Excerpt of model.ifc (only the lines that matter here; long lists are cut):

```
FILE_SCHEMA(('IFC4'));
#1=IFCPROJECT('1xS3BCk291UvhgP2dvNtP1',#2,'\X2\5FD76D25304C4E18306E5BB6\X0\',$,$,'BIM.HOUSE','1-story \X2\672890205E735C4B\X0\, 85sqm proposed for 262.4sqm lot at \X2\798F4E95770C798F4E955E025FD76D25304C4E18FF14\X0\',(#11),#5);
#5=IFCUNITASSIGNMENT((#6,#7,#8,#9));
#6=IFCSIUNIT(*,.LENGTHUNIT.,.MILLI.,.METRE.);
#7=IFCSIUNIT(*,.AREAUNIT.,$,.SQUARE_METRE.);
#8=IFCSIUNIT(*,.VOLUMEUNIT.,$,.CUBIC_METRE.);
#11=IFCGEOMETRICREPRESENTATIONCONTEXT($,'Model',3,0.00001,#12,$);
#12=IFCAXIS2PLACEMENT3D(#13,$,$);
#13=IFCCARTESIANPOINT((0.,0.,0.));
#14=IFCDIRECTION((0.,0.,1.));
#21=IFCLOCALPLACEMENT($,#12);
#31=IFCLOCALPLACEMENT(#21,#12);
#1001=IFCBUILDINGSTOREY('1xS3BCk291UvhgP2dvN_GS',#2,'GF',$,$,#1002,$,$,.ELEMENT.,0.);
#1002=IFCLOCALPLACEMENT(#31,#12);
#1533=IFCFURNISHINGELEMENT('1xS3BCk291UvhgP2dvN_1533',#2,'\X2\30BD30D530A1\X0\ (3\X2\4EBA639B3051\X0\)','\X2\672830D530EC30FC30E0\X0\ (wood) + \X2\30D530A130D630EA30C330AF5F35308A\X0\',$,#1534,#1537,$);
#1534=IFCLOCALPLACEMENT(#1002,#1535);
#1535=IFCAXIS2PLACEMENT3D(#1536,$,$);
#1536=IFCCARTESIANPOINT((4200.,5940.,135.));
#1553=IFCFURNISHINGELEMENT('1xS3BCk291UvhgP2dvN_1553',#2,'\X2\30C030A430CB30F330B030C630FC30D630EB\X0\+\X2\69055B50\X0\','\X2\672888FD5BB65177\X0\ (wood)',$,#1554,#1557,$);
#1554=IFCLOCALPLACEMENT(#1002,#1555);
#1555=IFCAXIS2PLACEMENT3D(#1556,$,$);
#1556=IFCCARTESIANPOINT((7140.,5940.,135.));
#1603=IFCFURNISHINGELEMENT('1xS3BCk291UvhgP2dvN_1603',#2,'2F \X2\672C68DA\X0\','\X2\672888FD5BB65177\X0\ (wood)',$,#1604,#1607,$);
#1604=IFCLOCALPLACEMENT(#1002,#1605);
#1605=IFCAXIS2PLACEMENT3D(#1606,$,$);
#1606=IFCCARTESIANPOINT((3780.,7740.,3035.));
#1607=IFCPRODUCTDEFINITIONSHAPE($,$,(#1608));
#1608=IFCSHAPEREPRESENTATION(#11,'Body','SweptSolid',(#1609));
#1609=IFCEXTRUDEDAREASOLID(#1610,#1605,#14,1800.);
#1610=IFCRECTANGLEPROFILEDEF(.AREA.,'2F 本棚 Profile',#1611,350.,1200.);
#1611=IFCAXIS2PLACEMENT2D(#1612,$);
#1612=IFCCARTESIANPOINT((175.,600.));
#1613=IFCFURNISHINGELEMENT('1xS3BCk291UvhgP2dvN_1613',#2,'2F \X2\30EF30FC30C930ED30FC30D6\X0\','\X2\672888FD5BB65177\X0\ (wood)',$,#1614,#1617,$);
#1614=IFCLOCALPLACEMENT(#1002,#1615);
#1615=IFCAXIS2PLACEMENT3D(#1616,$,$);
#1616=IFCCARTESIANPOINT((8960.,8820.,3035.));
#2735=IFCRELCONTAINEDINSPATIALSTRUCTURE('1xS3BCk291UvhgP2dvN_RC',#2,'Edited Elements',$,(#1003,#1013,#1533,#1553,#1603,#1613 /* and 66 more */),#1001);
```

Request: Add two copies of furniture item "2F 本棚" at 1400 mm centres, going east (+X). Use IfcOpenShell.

```python
import numpy as np
import ifcopenshell
import ifcopenshell.api.geometry
import ifcopenshell.api.root
import ifcopenshell.util.element
import ifcopenshell.util.placement
import ifcopenshell.util.unit

model = ifcopenshell.open("model.ifc")
unit_scale = ifcopenshell.util.unit.calculate_unit_scale(model)


def reuse_history(source, copy):
    """copy_class also copies each property set's owner history, people and application; keep the originals."""
    for rel in copy.IsDefinedBy:
        if rel.is_a("IfcRelDefinesByProperties") and (history := rel.RelatingPropertyDefinition.OwnerHistory):
            rel.RelatingPropertyDefinition.OwnerHistory = source.OwnerHistory
            ifcopenshell.util.element.remove_deep2(model, history)


source = model.by_guid("1xS3BCk291UvhgP2dvN_1603")
base = ifcopenshell.util.placement.get_local_placement(source.ObjectPlacement)
step = np.array([1.0, 0.0, 0.0]) * 1.4 / unit_scale

for i in range(1, 3):
    copy = ifcopenshell.api.root.copy_class(model, product=source)
    copy.Representation = ifcopenshell.util.element.copy_deep(
        model, source.Representation, exclude=["IfcGeometricRepresentationContext", "IfcRepresentationMap"]
    )
    reuse_history(source, copy)
    matrix = base.copy()
    matrix[:3, 3] += i * step
    print("added at", matrix[:3, 3].round(3) + 0.0)
    ifcopenshell.api.geometry.edit_object_placement(model, product=copy, matrix=matrix, is_si=False)

model.write("model-out.ifc")
```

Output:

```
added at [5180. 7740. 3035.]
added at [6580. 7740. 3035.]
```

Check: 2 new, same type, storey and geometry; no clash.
